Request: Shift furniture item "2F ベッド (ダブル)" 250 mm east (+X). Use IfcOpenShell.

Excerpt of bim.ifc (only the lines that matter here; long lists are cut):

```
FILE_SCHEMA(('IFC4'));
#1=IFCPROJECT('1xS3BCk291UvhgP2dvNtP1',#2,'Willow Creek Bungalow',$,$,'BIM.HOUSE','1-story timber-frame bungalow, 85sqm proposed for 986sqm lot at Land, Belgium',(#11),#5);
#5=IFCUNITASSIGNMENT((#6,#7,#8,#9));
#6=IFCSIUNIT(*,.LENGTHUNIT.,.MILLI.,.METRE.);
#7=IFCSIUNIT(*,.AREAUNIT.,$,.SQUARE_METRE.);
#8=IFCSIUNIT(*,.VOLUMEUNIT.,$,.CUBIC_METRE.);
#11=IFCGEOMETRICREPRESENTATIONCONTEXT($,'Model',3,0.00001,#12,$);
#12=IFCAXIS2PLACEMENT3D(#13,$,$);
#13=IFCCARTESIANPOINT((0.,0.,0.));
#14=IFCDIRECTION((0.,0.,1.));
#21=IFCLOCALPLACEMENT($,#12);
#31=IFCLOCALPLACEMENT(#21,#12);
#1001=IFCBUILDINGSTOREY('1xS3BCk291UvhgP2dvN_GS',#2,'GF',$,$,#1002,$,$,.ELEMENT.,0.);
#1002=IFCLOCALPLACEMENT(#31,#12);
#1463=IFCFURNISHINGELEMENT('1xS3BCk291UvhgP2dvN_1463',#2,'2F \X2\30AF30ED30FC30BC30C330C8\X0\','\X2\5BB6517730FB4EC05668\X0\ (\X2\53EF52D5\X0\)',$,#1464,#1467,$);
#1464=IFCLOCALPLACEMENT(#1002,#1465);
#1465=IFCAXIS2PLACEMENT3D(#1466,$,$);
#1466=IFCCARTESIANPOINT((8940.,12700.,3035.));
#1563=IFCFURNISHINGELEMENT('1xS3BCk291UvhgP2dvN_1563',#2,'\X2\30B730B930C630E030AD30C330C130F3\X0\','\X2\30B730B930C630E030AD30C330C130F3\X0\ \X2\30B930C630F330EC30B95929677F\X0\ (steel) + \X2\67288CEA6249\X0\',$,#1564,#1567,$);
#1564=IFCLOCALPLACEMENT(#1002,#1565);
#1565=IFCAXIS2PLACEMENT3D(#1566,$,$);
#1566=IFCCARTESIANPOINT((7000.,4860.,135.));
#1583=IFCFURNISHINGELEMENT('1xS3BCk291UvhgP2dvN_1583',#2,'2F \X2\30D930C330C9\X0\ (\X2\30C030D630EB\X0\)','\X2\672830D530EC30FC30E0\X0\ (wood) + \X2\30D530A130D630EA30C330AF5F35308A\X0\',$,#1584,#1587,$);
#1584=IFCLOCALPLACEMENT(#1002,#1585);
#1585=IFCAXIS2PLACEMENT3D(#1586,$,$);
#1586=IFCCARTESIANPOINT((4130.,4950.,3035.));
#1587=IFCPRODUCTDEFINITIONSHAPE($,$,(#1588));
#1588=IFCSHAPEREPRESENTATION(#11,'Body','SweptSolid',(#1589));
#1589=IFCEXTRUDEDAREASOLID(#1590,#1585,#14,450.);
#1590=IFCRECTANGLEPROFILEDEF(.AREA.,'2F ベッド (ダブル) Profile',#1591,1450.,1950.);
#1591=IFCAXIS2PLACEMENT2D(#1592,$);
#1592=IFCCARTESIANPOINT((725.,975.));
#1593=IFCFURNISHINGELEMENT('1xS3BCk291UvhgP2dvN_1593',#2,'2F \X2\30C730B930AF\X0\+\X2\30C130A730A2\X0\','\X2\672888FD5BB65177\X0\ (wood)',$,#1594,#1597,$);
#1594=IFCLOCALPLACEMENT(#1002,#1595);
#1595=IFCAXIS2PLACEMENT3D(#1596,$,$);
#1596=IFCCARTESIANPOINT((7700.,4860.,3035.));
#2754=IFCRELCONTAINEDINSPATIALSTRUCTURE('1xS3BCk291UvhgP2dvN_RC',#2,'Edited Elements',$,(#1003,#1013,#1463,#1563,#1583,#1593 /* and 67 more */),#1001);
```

```python
import ifcopenshell
import ifcopenshell.api.geometry
import ifcopenshell.util.placement
import ifcopenshell.util.unit

model = ifcopenshell.open("bim.ifc")
unit_scale = ifcopenshell.util.unit.calculate_unit_scale(model)

item = model.by_guid("1xS3BCk291UvhgP2dvN_1583")
matrix = ifcopenshell.util.placement.get_local_placement(item.ObjectPlacement)
matrix[0, 3] += 0.25 / unit_scale
ifcopenshell.api.geometry.edit_object_placement(model, product=item, matrix=matrix, is_si=False)

print(ifcopenshell.util.placement.get_local_placement(item.ObjectPlacement).round(3) + 0.0)

model.write("bim_v2.ifc")
```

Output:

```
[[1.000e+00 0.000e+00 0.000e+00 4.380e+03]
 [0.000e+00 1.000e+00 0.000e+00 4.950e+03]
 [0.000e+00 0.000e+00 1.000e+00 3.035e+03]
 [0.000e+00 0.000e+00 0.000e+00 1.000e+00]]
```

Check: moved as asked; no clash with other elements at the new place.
